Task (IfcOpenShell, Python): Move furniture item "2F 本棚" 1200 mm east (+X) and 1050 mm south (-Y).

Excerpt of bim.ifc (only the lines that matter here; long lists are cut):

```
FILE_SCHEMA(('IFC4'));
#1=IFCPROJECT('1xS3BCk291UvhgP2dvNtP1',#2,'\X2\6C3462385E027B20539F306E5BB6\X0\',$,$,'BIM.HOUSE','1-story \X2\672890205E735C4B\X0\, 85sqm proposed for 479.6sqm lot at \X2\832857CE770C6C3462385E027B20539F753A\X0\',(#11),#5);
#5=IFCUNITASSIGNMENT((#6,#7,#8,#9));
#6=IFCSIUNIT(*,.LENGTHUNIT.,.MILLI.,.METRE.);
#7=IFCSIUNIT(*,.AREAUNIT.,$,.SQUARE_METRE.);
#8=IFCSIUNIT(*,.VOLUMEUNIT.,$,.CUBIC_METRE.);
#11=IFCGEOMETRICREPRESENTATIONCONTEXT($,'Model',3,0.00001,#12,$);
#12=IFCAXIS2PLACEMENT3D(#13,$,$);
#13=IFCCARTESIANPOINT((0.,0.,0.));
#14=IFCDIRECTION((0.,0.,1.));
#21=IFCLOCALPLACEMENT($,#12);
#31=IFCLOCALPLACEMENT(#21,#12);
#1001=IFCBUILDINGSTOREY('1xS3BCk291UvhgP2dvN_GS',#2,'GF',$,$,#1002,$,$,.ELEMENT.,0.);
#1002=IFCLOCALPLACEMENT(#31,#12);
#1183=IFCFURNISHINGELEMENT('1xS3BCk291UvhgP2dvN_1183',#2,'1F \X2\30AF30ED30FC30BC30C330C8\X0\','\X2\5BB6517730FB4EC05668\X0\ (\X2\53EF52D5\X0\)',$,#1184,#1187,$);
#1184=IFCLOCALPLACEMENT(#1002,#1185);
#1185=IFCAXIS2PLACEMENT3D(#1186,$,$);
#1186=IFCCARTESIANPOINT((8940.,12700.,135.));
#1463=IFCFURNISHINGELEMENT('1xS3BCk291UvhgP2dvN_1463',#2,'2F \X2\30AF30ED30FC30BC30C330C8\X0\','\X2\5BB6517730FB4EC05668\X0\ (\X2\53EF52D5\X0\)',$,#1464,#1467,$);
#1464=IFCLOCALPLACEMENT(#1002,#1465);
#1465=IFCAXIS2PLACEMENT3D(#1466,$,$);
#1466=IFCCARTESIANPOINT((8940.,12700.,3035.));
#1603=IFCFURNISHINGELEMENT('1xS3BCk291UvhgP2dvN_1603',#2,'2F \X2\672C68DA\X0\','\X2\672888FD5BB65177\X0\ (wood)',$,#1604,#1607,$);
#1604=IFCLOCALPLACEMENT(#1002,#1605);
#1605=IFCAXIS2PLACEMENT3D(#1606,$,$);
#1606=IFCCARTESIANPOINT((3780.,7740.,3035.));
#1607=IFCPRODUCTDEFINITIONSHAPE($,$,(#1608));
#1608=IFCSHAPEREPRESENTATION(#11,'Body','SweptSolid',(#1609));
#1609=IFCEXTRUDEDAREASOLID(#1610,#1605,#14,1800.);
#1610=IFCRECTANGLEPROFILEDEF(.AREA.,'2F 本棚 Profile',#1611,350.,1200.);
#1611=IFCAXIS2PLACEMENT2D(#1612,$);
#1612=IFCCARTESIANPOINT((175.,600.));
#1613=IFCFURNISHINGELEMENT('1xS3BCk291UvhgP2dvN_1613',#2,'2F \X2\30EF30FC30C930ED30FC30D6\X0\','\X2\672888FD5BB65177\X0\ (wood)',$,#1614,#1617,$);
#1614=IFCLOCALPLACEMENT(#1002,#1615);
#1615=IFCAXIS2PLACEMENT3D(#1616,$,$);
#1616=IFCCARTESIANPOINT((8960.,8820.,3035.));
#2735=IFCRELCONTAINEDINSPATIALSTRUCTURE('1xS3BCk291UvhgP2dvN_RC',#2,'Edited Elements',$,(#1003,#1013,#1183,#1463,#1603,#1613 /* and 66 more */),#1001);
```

```python
import ifcopenshell
import ifcopenshell.api.geometry
import ifcopenshell.util.placement

model = ifcopenshell.open("bim.ifc")

item = model.by_guid("1xS3BCk291UvhgP2dvN_1603")
matrix = ifcopenshell.util.placement.get_local_placement(item.ObjectPlacement)
matrix[0, 3] += 1200.0
matrix[1, 3] -= 1050.0
ifcopenshell.api.geometry.edit_object_placement(model, product=item, matrix=matrix, is_si=False)

print(ifcopenshell.util.placement.get_local_placement(item.ObjectPlacement).round(3) + 0.0)

model.write("bim_v2.ifc")
```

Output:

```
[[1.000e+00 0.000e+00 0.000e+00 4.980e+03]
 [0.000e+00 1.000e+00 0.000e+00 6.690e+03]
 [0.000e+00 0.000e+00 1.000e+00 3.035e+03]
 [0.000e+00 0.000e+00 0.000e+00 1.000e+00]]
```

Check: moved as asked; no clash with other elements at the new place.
